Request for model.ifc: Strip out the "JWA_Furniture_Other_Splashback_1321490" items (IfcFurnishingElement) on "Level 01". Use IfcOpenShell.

First a look at what the model holds.

```python
import ifcopenshell
import ifcopenshell.util.element

model = ifcopenshell.open("model.ifc")
print(model.schema)
storey = next(s for s in model.by_type("IfcBuildingStorey") if s.Name == "Level 01")
furniture = [e for e in ifcopenshell.util.element.get_decomposition(storey) if e.is_a("IfcFurnishingElement")]
seen = {}
for e in furniture:
    element_type = ifcopenshell.util.element.get_type(e)
    name = element_type.Name if element_type not in (None, e) else None
    seen[name] = seen.get(name, 0) + 1
for name, count in sorted(seen.items(), key=str):
    print(count, "x", name)
```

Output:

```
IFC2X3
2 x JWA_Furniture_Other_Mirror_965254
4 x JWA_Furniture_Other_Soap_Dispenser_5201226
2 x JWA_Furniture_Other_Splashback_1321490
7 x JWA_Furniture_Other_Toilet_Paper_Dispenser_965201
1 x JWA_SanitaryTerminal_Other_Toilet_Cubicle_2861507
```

```python
import ifcopenshell
import ifcopenshell.api.root
import ifcopenshell.util.element

model = ifcopenshell.open("model.ifc")

storey = next(s for s in model.by_type("IfcBuildingStorey") if s.Name == "Level 01")
furniture = [e for e in ifcopenshell.util.element.get_decomposition(storey) if e.is_a("IfcFurnishingElement")]
targets = [e for e in furniture if (t := ifcopenshell.util.element.get_type(e)) not in (None, e) and t.Name == "JWA_Furniture_Other_Splashback_1321490"]

for e in targets:
    ifcopenshell.api.root.remove_product(model, product=e)
print(len(targets), "removed")

model.write("model_v2.ifc")
```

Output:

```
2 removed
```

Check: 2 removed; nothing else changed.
